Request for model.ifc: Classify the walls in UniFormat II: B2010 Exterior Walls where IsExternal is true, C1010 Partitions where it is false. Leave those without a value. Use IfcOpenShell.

First a look at what the model holds.

```python
import ifcopenshell
import ifcopenshell.util.element

model = ifcopenshell.open("model.ifc")
print(model.schema)
print("classifications:", [c.Name for c in model.by_type("IfcClassification")])
values = [ifcopenshell.util.element.get_pset(e, "Pset_WallCommon", "IsExternal") for e in model.by_type("IfcWall")]
for value in (True, False, None):
    print("IsExternal", value, values.count(value))
```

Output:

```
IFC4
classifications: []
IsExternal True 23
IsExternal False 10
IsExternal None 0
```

```python
import ifcopenshell
import ifcopenshell.api.classification
import ifcopenshell.util.element

model = ifcopenshell.open("model.ifc")

system = ifcopenshell.api.classification.add_classification(model, classification="UniFormat II")

walls = model.by_type("IfcWall")
external = {e: ifcopenshell.util.element.get_pset(e, "Pset_WallCommon", "IsExternal") for e in walls}
for flag, code, name in ((True, "B2010", "Exterior Walls"), (False, "C1010", "Partitions")):
    products = [e for e in walls if external[e] is flag]
    ifcopenshell.api.classification.add_reference(
        model, products=products, classification=system, identification=code, name=name
    )
    print(code, len(products))

model.write("model_updated.ifc")
```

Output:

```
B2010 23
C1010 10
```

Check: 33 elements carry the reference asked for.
